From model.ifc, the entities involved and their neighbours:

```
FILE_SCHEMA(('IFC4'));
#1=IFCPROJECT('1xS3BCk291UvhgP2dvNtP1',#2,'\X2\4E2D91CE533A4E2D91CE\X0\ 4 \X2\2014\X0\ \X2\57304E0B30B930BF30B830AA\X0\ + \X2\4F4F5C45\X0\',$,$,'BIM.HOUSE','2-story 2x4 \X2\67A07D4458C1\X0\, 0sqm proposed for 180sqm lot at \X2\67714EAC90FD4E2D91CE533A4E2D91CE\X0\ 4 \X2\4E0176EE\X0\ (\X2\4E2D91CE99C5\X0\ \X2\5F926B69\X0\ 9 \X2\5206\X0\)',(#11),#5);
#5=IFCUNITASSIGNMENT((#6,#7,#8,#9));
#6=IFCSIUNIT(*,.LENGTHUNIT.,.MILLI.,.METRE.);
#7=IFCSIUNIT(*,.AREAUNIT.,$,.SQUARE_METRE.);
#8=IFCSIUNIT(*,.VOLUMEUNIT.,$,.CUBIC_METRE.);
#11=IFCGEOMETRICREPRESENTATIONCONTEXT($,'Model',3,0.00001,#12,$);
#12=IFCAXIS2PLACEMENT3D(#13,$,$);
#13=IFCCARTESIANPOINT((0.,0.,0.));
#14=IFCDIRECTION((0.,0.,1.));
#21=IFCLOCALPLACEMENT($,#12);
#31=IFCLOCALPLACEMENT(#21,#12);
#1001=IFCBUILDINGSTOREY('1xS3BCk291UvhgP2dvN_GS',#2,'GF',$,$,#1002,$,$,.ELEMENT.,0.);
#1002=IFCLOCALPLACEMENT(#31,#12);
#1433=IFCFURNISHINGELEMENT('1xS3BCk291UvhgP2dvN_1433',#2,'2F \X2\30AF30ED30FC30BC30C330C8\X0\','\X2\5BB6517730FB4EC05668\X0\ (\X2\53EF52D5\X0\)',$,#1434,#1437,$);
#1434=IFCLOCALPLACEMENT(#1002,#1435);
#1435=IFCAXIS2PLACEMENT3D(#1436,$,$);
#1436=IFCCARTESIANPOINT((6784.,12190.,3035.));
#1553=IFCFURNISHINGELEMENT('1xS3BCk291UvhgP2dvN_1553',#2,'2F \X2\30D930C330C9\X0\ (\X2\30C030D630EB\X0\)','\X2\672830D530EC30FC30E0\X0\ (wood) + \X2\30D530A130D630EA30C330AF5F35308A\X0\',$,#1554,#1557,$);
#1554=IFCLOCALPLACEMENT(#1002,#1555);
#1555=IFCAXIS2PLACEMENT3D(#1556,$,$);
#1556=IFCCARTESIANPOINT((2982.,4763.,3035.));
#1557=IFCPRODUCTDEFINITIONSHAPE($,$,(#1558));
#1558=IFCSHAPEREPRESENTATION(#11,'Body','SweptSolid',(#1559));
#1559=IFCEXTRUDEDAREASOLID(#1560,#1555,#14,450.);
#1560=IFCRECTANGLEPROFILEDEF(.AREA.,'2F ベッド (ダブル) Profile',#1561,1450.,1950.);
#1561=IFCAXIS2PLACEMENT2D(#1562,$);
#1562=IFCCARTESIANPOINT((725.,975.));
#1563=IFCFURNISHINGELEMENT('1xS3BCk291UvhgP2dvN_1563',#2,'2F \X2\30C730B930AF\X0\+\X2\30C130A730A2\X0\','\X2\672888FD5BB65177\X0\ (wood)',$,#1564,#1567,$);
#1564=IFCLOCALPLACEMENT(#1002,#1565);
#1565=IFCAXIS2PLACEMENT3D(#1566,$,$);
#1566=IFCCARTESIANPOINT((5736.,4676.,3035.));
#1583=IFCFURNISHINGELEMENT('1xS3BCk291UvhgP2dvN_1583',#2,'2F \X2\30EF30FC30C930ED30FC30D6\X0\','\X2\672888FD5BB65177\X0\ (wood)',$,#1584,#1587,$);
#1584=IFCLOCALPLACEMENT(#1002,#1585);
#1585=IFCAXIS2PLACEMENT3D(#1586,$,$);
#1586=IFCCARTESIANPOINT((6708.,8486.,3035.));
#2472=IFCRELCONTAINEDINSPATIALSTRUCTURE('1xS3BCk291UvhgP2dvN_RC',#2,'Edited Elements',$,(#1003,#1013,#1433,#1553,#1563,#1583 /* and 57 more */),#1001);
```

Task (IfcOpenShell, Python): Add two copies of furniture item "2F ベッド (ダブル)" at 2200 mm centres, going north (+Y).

```python
import numpy as np
import ifcopenshell
import ifcopenshell.api.geometry
import ifcopenshell.api.root
import ifcopenshell.util.element
import ifcopenshell.util.placement
import ifcopenshell.util.unit

model = ifcopenshell.open("model.ifc")
unit_scale = ifcopenshell.util.unit.calculate_unit_scale(model)


def reuse_history(source, copy):
    """copy_class also copies each property set's owner history, people and application; keep the originals."""
    for rel in copy.IsDefinedBy:
        if rel.is_a("IfcRelDefinesByProperties") and (history := rel.RelatingPropertyDefinition.OwnerHistory):
            rel.RelatingPropertyDefinition.OwnerHistory = source.OwnerHistory
            ifcopenshell.util.element.remove_deep2(model, history)


source = model.by_guid("1xS3BCk291UvhgP2dvN_1553")
base = ifcopenshell.util.placement.get_local_placement(source.ObjectPlacement)
step = np.array([0.0, 1.0, 0.0]) * 2.2 / unit_scale

for i in range(1, 3):
    copy = ifcopenshell.api.root.copy_class(model, product=source)
    copy.Representation = ifcopenshell.util.element.copy_deep(
        model, source.Representation, exclude=["IfcGeometricRepresentationContext", "IfcRepresentationMap"]
    )
    reuse_history(source, copy)
    matrix = base.copy()
    matrix[:3, 3] += i * step
    print("added at", matrix[:3, 3].round(3) + 0.0)
    ifcopenshell.api.geometry.edit_object_placement(model, product=copy, matrix=matrix, is_si=False)

model.write("model_rev.ifc")
```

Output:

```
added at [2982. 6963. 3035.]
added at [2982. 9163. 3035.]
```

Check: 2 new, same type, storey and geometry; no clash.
